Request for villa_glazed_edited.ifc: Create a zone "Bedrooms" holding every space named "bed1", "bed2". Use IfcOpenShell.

First a look at what the model holds.

```python
import ifcopenshell

model = ifcopenshell.open("villa_glazed_edited.ifc")
print(model.schema)
seen = {}
for space in model.by_type("IfcSpace"):
    seen[space.LongName] = seen.get(space.LongName, 0) + 1
for name, count in sorted(seen.items(), key=str):
    print(count, "x", name)
print("zones:", [z.Name for z in model.by_type("IfcZone")][:20])
```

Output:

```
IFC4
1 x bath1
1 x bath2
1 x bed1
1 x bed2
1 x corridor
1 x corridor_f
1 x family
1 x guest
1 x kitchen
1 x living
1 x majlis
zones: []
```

```python
import ifcopenshell
import ifcopenshell.api.group
import ifcopenshell.api.root

model = ifcopenshell.open("villa_glazed_edited.ifc")

names = {"bed1", "bed2"}
spaces = [s for s in model.by_type("IfcSpace") if s.LongName in names]

zone = ifcopenshell.api.root.create_entity(model, ifc_class="IfcZone", name="Bedrooms")
ifcopenshell.api.group.assign_group(model, products=spaces, group=zone)
print(len(spaces), "spaces in", zone.Name)

model.write("villa_glazed_edited-out.ifc")
```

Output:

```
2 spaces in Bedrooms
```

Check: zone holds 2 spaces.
